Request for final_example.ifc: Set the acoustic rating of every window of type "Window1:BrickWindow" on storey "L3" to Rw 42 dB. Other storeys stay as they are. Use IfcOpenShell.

First a look at what the model holds.

```python
import ifcopenshell
import ifcopenshell.util.element

model = ifcopenshell.open("final_example.ifc")
print(model.schema)
storey = next(s for s in model.by_type("IfcBuildingStorey") if s.Name == "L3")
windows = [e for e in ifcopenshell.util.element.get_decomposition(storey) if e.is_a("IfcWindow")]
seen = {}
for e in windows:
    element_type = ifcopenshell.util.element.get_type(e)
    key = (element_type.Name if element_type != e and element_type else None, ifcopenshell.util.element.get_pset(e, "Pset_WindowCommon", "AcousticRating"))
    seen[key] = seen.get(key, 0) + 1
for (name, value), count in sorted(seen.items(), key=str):
    print(count, "x", name, "|", value)
```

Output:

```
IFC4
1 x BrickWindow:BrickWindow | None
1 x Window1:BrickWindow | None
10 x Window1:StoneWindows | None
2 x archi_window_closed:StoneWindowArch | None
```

```python
import ifcopenshell
import ifcopenshell.api.pset
import ifcopenshell.util.element

model = ifcopenshell.open("final_example.ifc")

storey = next(s for s in model.by_type("IfcBuildingStorey") if s.Name == "L3")
windows = [e for e in ifcopenshell.util.element.get_decomposition(storey) if e.is_a("IfcWindow")]

count = 0
for e in windows:
    element_type = ifcopenshell.util.element.get_type(e)
    if element_type in (None, e) or element_type.Name != "Window1:BrickWindow":
        continue
    # add_pset returns the element's existing set when there is one.
    pset = ifcopenshell.api.pset.add_pset(model, product=e, name="Pset_WindowCommon")
    ifcopenshell.api.pset.edit_pset(model, pset=pset, properties={"AcousticRating": "Rw 42 dB"})
    count += 1

print(count, "windows updated")

model.write("final_example-out.ifc")
```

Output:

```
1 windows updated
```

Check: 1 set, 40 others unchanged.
